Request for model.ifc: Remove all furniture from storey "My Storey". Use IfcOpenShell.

First a look at what the model holds.

```python
import ifcopenshell
import ifcopenshell.util.element

model = ifcopenshell.open("model.ifc")
print(model.schema)
storey = next(s for s in model.by_type("IfcBuildingStorey") if s.Name == "My Storey")
furniture = [e for e in ifcopenshell.util.element.get_decomposition(storey) if e.is_a("IfcFurnishingElement")]
seen = {}
for e in furniture:
    element_type = ifcopenshell.util.element.get_type(e)
    name = element_type.Name if element_type not in (None, e) else None
    seen[name] = seen.get(name, 0) + 1
for name, count in sorted(seen.items(), key=str):
    print(count, "x", name)
```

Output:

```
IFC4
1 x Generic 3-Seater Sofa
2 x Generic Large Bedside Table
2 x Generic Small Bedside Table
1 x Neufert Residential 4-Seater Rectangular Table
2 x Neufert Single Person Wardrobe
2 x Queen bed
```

```python
import ifcopenshell
import ifcopenshell.api.root
import ifcopenshell.util.element

model = ifcopenshell.open("model.ifc")

storey = next(s for s in model.by_type("IfcBuildingStorey") if s.Name == "My Storey")
furniture = [e for e in ifcopenshell.util.element.get_decomposition(storey) if e.is_a("IfcFurnishingElement")]

for e in furniture:
    ifcopenshell.api.root.remove_product(model, product=e)
print(len(furniture), "removed")

model.write("model-out.ifc")
```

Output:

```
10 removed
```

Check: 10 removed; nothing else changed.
